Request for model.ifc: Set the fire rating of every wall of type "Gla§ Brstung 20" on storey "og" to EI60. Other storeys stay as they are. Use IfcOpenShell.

First a look at what the model holds.

```python
import ifcopenshell
import ifcopenshell.util.element

model = ifcopenshell.open("model.ifc")
print(model.schema)
storey = next(s for s in model.by_type("IfcBuildingStorey") if s.Name == "og")
walls = [e for e in ifcopenshell.util.element.get_decomposition(storey) if e.is_a("IfcWall")]
seen = {}
for e in walls:
    element_type = ifcopenshell.util.element.get_type(e)
    key = (element_type.Name if element_type != e and element_type else None, ifcopenshell.util.element.get_pset(e, "Pset_WallCommon", "FireRating"))
    seen[key] = seen.get(key, 0) + 1
for (name, value), count in sorted(seen.items(), key=str):
    print(count, "x", name, "|", value)
```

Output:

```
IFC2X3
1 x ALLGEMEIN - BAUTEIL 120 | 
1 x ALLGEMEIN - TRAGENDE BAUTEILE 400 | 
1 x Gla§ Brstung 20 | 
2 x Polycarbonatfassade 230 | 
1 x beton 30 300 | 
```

```python
import ifcopenshell
import ifcopenshell.api.pset
import ifcopenshell.util.element

model = ifcopenshell.open("model.ifc")

storey = next(s for s in model.by_type("IfcBuildingStorey") if s.Name == "og")
walls = [e for e in ifcopenshell.util.element.get_decomposition(storey) if e.is_a("IfcWall")]

count = 0
for e in walls:
    element_type = ifcopenshell.util.element.get_type(e)
    if element_type in (None, e) or element_type.Name != 'Gla§ Br\x9fstung 20':
        continue
    # add_pset returns the element's existing set when there is one.
    pset = ifcopenshell.api.pset.add_pset(model, product=e, name="Pset_WallCommon")
    ifcopenshell.api.pset.edit_pset(model, pset=pset, properties={"FireRating": "EI60"})
    count += 1

print(count, "walls updated")

model.write("model_updated.ifc")
```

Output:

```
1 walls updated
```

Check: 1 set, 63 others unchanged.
